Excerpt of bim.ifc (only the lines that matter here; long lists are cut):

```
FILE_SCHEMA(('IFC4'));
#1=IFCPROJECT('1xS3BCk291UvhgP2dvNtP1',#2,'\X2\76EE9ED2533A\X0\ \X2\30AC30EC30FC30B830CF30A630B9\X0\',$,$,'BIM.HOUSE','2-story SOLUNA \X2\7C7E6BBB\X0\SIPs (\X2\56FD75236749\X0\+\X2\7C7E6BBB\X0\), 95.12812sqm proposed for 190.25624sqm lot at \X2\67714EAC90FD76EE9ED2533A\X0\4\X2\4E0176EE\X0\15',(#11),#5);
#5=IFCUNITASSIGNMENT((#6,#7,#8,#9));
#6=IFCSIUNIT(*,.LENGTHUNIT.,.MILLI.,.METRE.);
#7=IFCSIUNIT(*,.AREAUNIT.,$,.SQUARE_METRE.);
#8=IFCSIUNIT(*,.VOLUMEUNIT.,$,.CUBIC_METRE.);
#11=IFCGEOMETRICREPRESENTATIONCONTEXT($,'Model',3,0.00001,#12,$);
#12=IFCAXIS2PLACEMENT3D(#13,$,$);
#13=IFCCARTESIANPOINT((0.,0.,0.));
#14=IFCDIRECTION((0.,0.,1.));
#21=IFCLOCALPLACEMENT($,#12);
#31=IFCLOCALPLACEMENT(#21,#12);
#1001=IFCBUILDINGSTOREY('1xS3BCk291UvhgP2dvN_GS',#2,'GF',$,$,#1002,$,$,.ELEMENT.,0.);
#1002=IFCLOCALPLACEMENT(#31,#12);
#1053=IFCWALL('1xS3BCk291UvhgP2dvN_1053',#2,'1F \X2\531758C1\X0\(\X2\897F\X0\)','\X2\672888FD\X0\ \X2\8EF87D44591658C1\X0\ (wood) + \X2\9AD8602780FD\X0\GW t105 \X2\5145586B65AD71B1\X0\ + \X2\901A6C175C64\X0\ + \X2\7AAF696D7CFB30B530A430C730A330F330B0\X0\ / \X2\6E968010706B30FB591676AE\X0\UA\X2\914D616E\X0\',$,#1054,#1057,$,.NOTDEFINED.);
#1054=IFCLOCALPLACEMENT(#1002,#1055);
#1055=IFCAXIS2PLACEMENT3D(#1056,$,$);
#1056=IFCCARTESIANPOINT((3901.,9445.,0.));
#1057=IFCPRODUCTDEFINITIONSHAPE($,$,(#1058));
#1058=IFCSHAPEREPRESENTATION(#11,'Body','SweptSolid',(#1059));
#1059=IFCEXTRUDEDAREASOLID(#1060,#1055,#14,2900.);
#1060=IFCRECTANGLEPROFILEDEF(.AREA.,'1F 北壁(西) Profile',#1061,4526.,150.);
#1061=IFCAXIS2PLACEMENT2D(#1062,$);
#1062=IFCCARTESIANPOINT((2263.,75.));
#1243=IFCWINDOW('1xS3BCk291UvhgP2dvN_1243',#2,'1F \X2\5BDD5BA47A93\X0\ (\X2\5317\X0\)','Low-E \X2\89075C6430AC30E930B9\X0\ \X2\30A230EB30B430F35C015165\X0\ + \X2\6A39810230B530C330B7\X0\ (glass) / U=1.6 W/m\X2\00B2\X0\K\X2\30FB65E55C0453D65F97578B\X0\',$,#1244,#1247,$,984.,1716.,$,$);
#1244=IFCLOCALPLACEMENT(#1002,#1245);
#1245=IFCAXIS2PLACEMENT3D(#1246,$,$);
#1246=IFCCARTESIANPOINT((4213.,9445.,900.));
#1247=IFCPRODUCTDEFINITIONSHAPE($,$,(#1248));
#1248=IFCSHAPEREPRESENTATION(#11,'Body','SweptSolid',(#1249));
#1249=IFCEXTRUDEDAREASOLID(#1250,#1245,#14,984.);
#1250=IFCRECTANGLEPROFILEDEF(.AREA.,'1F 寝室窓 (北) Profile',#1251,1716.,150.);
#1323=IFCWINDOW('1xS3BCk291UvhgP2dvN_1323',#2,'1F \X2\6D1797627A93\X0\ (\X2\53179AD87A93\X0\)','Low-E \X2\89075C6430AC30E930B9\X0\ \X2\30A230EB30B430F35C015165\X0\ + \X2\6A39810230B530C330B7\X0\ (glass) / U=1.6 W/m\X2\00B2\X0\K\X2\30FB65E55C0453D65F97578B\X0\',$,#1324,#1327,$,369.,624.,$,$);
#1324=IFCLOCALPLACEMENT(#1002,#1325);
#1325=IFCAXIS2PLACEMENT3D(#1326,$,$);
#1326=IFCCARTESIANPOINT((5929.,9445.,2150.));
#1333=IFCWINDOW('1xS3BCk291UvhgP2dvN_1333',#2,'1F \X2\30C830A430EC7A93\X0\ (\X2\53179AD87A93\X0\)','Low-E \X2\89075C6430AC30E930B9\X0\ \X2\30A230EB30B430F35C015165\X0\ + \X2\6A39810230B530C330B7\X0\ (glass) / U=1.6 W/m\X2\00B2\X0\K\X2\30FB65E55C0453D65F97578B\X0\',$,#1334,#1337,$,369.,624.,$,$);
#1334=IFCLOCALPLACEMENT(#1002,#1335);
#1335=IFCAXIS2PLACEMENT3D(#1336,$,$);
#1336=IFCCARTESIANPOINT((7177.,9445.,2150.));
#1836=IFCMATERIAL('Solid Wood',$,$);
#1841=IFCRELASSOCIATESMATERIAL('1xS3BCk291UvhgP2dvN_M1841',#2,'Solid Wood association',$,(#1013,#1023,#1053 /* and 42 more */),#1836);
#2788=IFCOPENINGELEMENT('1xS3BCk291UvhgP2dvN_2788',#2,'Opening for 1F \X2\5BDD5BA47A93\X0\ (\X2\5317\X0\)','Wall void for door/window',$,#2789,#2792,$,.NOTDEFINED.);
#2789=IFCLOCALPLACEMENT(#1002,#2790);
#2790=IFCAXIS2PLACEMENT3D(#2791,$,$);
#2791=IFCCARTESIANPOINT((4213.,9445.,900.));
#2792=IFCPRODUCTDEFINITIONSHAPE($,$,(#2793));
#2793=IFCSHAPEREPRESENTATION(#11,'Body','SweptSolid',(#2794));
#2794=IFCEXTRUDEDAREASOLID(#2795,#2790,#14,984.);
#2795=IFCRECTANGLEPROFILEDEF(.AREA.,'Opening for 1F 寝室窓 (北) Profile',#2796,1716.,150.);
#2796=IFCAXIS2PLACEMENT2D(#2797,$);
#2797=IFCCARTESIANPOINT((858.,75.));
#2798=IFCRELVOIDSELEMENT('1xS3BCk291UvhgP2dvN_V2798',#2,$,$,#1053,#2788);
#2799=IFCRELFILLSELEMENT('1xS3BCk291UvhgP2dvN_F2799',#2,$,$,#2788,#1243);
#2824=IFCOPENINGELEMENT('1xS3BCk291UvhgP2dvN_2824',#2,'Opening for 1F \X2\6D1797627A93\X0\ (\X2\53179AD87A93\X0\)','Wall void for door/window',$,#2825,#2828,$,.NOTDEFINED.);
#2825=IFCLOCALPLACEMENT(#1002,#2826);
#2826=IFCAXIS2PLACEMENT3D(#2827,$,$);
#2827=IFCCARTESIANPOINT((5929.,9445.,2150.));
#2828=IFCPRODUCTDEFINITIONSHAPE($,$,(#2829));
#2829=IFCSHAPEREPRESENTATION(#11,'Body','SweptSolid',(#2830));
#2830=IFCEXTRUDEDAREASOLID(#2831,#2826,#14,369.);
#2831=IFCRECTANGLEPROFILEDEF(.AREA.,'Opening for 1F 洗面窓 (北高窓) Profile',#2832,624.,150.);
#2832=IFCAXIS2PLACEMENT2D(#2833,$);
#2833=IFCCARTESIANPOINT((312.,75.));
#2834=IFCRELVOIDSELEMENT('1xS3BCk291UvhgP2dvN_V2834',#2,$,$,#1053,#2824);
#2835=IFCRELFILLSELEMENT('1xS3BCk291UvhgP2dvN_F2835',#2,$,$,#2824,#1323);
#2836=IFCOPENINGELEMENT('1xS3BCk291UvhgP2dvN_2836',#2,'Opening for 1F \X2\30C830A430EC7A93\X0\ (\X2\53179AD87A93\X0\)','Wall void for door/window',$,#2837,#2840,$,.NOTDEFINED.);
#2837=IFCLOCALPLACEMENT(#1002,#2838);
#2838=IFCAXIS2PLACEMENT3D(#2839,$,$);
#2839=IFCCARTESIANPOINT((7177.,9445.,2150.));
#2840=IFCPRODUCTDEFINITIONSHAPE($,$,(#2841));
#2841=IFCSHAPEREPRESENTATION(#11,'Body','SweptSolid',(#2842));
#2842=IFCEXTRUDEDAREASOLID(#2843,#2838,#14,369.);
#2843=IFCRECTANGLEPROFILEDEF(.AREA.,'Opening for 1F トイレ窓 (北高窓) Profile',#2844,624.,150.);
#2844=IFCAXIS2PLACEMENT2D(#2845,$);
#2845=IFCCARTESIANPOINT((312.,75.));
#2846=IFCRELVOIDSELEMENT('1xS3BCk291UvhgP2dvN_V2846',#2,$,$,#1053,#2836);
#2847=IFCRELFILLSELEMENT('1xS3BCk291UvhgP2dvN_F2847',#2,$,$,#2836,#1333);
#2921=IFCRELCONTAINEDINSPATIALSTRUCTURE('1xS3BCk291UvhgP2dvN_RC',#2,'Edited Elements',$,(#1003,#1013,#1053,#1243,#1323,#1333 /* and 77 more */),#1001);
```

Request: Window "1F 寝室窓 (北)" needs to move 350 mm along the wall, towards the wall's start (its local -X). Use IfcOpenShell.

```python
import ifcopenshell
import ifcopenshell.api.geometry
import ifcopenshell.util.placement

model = ifcopenshell.open("bim.ifc")

window = model.by_guid("1xS3BCk291UvhgP2dvN_1243")
opening = window.FillsVoids[0].RelatingOpeningElement
wall = opening.VoidsElements[0].RelatingBuildingElement

wall_matrix = ifcopenshell.util.placement.get_local_placement(wall.ObjectPlacement)
shift = wall_matrix[:3, 0] * -350.0
before = ifcopenshell.util.placement.get_local_placement(window.ObjectPlacement)[:3, 3].copy()

# The window is not placed relative to its opening, so move both.
for product in (opening, window):
    matrix = ifcopenshell.util.placement.get_local_placement(product.ObjectPlacement)
    matrix[:3, 3] += shift
    ifcopenshell.api.geometry.edit_object_placement(model, product=product, matrix=matrix, is_si=False)

after = ifcopenshell.util.placement.get_local_placement(window.ObjectPlacement)[:3, 3]
print("window moved by", (after - before).round(3) + 0.0)

model.write("bim_edited.ifc")
```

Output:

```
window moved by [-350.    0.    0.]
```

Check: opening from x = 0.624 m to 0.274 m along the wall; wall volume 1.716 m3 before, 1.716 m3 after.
